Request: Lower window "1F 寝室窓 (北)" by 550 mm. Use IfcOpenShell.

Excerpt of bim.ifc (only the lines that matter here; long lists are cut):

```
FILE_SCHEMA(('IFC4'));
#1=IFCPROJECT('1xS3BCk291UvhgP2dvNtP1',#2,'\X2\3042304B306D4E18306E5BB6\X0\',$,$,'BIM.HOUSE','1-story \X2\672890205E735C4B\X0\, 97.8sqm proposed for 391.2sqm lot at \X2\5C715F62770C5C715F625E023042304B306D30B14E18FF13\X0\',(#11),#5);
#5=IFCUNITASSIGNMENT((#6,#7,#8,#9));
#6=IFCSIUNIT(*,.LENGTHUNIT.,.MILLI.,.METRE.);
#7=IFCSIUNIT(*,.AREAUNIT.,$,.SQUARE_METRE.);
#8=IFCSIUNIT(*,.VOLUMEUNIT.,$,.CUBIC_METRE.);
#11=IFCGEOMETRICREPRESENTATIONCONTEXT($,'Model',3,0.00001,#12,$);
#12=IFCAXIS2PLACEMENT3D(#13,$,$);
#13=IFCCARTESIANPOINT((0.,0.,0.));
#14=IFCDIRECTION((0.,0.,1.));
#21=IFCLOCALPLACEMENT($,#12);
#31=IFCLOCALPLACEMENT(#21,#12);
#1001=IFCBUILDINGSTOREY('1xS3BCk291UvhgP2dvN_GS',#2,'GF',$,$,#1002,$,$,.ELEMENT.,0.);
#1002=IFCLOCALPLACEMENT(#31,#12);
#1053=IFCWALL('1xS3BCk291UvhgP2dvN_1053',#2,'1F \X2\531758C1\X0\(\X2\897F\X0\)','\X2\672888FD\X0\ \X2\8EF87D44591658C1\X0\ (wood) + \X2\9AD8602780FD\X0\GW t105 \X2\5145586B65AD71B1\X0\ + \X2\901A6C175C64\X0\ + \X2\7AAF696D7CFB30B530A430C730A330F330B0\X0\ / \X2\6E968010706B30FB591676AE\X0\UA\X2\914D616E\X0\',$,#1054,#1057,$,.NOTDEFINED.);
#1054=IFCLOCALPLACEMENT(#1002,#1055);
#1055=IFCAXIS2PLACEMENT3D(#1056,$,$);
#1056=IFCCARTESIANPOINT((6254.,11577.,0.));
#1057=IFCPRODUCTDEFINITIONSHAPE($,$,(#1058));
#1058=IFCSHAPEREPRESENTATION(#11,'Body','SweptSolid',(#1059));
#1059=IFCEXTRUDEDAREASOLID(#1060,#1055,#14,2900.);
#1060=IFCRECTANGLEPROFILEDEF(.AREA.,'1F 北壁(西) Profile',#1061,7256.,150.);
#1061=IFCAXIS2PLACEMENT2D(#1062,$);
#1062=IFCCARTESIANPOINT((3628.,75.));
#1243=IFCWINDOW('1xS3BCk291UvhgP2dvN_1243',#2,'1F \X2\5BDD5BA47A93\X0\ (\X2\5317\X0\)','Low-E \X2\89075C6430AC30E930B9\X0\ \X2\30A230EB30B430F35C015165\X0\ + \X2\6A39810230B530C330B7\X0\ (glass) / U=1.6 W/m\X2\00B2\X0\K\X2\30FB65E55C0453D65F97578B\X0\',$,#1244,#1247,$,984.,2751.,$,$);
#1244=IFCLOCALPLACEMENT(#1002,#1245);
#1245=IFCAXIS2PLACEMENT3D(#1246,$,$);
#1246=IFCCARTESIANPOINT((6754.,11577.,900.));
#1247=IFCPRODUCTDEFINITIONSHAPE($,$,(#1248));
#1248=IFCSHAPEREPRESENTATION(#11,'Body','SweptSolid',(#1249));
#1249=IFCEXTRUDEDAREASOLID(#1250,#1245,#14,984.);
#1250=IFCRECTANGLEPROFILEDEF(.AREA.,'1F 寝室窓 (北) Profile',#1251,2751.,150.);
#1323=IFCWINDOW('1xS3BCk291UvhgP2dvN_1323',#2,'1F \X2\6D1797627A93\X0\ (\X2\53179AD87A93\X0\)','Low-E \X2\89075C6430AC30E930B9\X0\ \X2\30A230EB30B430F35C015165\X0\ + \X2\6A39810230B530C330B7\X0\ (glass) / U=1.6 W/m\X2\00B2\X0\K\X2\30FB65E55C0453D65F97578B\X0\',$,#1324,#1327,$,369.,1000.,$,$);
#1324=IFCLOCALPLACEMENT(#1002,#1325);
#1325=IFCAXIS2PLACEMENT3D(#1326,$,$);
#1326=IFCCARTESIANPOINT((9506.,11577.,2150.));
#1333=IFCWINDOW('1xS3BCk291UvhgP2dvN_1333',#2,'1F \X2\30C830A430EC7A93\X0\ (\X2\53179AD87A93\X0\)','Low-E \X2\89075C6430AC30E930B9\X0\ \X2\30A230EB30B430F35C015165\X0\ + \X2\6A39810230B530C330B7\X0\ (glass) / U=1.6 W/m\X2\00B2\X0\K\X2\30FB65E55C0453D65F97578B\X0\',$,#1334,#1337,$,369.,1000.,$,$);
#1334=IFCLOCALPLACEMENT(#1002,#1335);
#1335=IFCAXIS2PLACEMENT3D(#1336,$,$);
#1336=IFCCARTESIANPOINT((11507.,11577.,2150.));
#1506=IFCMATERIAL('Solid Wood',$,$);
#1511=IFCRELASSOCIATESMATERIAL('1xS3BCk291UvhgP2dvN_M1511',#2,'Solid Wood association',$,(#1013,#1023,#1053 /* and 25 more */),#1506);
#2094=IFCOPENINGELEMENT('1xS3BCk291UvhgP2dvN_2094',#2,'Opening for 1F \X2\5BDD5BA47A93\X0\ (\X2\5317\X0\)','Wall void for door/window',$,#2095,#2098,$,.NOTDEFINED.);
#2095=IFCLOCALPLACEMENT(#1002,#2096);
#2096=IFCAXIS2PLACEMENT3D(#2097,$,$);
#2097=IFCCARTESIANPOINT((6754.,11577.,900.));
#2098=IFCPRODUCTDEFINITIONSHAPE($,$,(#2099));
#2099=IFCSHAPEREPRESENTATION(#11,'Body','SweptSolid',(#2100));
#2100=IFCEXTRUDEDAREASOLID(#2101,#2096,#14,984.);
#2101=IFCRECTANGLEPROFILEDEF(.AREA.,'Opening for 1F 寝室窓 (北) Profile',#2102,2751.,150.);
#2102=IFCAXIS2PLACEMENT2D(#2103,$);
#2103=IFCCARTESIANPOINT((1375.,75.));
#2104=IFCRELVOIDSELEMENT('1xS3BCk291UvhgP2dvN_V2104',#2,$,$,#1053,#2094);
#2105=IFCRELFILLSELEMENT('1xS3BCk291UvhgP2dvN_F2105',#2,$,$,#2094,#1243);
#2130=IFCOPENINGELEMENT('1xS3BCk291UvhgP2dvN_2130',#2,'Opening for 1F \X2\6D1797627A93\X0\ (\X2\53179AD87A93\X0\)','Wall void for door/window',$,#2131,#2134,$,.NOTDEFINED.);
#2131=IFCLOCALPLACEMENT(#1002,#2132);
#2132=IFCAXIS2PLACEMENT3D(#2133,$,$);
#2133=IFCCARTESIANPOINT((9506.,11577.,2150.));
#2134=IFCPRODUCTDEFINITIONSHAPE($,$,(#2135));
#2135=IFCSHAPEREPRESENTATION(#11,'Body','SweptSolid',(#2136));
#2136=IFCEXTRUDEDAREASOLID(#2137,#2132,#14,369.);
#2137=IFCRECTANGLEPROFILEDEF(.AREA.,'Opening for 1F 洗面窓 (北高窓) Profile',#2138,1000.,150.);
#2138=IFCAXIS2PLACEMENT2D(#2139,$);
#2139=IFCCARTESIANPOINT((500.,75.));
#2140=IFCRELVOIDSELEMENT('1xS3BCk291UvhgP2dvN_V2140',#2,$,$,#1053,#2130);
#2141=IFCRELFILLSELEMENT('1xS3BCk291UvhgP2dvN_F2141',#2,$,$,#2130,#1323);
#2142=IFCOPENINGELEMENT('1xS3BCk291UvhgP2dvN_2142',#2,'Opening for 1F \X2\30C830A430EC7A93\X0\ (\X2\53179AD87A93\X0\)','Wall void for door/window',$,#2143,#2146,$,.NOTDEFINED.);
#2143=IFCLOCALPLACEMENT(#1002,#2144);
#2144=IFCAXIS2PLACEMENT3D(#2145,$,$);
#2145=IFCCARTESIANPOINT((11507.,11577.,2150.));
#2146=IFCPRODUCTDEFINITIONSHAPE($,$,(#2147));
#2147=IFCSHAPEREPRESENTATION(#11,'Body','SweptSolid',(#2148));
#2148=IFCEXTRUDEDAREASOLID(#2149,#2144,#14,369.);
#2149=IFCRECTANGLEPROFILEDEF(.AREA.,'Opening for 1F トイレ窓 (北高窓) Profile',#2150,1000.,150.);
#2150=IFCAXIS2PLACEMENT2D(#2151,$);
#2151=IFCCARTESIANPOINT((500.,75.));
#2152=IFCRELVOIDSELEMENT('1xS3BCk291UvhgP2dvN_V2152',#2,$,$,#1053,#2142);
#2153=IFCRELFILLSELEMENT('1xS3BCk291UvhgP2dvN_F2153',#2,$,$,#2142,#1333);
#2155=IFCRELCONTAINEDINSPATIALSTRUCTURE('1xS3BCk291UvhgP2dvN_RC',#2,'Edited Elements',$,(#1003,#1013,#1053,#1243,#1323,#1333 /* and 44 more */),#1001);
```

```python
import numpy as np
import ifcopenshell
import ifcopenshell.api.geometry
import ifcopenshell.util.placement
import ifcopenshell.util.unit

model = ifcopenshell.open("bim.ifc")
unit_scale = ifcopenshell.util.unit.calculate_unit_scale(model)

window = model.by_id(1243)
opening = window.FillsVoids[0].RelatingOpeningElement
dz = -550.0

shift = np.array([0.0, 0.0, dz])
# The window is not placed relative to its opening, so move both.
for product in (opening, window):
    matrix = ifcopenshell.util.placement.get_local_placement(product.ObjectPlacement)
    matrix[:3, 3] += shift
    ifcopenshell.api.geometry.edit_object_placement(model, product=product, matrix=matrix, is_si=False)

print(f"moved by {dz * unit_scale:+.3f} m")

model.write("bim_edited.ifc")
```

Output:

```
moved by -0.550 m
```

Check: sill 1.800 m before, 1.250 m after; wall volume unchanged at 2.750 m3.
